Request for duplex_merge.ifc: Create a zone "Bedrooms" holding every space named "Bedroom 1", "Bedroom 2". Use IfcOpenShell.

First a look at what the model holds.

```python
import ifcopenshell

model = ifcopenshell.open("duplex_merge.ifc")
print(model.schema)
seen = {}
for space in model.by_type("IfcSpace"):
    seen[space.LongName] = seen.get(space.LongName, 0) + 1
for name, count in sorted(seen.items(), key=str):
    print(count, "x", name)
print("zones:", [z.Name for z in model.by_type("IfcZone")][:20])
```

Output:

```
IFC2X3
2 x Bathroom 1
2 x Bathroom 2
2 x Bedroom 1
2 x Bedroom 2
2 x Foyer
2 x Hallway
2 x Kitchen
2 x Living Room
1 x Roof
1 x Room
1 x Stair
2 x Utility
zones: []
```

```python
import ifcopenshell
import ifcopenshell.api.group
import ifcopenshell.api.root

model = ifcopenshell.open("duplex_merge.ifc")

names = {"Bedroom 1", "Bedroom 2"}
spaces = [s for s in model.by_type("IfcSpace") if s.LongName in names]

zone = ifcopenshell.api.root.create_entity(model, ifc_class="IfcZone", name="Bedrooms")
ifcopenshell.api.group.assign_group(model, products=spaces, group=zone)
print(len(spaces), "spaces in", zone.Name)

model.write("duplex_merge_updated.ifc")
```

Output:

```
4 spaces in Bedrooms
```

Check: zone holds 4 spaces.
